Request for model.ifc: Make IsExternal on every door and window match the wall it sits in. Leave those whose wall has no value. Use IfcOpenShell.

First a look at what the model holds.

```python
import ifcopenshell
import ifcopenshell.util.element

model = ifcopenshell.open("model.ifc")
print(model.schema)
seen = {}
for e in model.by_type("IfcDoor") + model.by_type("IfcWindow"):
    if not e.FillsVoids:
        continue
    host = e.FillsVoids[0].RelatingOpeningElement.VoidsElements[0].RelatingBuildingElement
    own = ifcopenshell.util.element.get_pset(e, f"Pset_{e.is_a()[3:].removesuffix('StandardCase')}Common", "IsExternal")
    wall = ifcopenshell.util.element.get_pset(host, "Pset_WallCommon", "IsExternal")
    seen[e.is_a(), own, wall] = seen.get((e.is_a(), own, wall), 0) + 1
for (cls, own, wall), count in sorted(seen.items(), key=str):
    print(count, cls, "IsExternal:", own, "| host wall:", wall)
```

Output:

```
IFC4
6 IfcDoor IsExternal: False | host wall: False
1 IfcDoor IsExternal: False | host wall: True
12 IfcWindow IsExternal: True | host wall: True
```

```python
import ifcopenshell
import ifcopenshell.api.pset
import ifcopenshell.util.element

model = ifcopenshell.open("model.ifc")

count = 0
for ifc_class, pset_name in (("IfcDoor", "Pset_DoorCommon"), ("IfcWindow", "Pset_WindowCommon")):
    for e in model.by_type(ifc_class):
        if not e.FillsVoids:
            continue
        host = e.FillsVoids[0].RelatingOpeningElement.VoidsElements[0].RelatingBuildingElement
        external = ifcopenshell.util.element.get_pset(host, "Pset_WallCommon", "IsExternal")
        if external is None or ifcopenshell.util.element.get_pset(e, pset_name, "IsExternal") == external:
            continue
        pset = ifcopenshell.api.pset.add_pset(model, product=e, name=pset_name)
        ifcopenshell.api.pset.edit_pset(model, pset=pset, properties={"IsExternal": external})
        count += 1

print(count, "updated")

model.write("model_rev.ifc")
```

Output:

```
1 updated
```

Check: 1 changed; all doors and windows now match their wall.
